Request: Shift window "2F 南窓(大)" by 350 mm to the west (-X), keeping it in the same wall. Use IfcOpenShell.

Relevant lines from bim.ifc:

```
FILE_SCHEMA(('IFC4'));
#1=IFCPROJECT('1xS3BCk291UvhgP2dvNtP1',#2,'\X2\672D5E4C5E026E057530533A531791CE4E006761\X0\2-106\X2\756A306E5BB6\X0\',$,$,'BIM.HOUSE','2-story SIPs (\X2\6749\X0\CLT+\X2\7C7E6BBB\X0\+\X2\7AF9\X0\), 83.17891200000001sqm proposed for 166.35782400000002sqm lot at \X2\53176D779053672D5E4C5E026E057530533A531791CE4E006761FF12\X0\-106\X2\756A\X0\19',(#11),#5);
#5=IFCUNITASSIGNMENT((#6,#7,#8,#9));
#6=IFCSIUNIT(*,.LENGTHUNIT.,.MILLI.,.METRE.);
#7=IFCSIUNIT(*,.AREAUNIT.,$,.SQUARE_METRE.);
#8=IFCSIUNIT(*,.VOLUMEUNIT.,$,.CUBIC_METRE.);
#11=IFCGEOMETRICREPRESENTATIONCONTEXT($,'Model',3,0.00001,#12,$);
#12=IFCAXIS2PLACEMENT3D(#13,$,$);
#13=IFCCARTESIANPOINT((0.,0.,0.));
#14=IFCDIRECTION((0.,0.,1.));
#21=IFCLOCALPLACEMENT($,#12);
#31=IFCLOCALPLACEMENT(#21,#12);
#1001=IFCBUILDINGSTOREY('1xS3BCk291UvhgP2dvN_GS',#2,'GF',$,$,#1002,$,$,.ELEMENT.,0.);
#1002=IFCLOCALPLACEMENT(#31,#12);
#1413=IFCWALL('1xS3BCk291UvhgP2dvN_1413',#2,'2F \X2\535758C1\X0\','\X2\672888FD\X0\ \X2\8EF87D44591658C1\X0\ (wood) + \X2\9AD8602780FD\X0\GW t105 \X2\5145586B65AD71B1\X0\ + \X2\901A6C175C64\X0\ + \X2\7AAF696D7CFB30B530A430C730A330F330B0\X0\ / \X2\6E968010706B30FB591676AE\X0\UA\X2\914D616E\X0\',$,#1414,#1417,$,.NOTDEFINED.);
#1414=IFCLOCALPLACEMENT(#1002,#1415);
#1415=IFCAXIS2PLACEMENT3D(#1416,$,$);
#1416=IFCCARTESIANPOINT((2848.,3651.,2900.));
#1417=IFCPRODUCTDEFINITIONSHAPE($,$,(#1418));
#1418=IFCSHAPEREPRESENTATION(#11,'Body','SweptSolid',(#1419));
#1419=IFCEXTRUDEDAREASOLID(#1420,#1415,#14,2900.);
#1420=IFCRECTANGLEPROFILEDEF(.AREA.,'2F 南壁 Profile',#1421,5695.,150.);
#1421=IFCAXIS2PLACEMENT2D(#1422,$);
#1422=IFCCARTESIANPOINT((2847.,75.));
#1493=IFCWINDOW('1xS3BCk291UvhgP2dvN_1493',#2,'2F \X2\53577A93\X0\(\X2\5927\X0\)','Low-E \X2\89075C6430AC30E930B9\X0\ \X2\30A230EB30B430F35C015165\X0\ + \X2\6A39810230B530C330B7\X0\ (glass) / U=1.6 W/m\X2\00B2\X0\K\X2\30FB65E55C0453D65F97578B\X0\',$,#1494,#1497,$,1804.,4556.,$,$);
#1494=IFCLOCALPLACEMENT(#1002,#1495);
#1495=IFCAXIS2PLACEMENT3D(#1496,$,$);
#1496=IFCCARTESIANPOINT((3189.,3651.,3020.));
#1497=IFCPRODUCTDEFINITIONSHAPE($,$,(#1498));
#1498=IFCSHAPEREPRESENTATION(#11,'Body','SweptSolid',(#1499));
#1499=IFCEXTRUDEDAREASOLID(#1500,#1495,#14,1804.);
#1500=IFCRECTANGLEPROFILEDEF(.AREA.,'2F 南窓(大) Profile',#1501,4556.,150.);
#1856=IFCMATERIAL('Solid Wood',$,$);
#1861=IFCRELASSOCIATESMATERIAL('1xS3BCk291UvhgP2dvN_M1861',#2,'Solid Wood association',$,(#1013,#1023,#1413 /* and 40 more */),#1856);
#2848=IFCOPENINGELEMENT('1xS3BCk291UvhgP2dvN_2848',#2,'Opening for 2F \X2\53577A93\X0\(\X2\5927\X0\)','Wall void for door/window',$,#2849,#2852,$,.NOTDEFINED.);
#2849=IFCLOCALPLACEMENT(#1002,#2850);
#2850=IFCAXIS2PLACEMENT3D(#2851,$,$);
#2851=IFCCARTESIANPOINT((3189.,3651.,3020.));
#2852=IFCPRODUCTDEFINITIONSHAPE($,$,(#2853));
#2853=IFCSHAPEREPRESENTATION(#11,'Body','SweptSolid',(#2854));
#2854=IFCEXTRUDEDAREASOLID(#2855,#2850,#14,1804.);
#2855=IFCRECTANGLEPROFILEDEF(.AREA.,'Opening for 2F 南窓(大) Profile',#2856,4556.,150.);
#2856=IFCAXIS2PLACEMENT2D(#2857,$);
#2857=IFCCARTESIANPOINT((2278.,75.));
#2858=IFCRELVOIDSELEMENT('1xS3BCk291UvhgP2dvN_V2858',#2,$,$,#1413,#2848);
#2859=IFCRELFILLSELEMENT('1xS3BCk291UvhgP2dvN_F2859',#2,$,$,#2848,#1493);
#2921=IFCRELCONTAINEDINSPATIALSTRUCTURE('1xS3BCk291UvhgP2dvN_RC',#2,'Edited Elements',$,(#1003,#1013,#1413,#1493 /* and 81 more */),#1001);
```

```python
import ifcopenshell
import ifcopenshell.api.geometry
import ifcopenshell.util.placement

model = ifcopenshell.open("bim.ifc")

window = model.by_guid("1xS3BCk291UvhgP2dvN_1493")
opening = window.FillsVoids[0].RelatingOpeningElement
wall = opening.VoidsElements[0].RelatingBuildingElement

wall_matrix = ifcopenshell.util.placement.get_local_placement(wall.ObjectPlacement)
shift = wall_matrix[:3, 0] * -350.0
before = ifcopenshell.util.placement.get_local_placement(window.ObjectPlacement)[:3, 3].copy()

# The window is not placed relative to its opening, so move both.
for product in (opening, window):
    matrix = ifcopenshell.util.placement.get_local_placement(product.ObjectPlacement)
    matrix[:3, 3] += shift
    ifcopenshell.api.geometry.edit_object_placement(model, product=product, matrix=matrix, is_si=False)

after = ifcopenshell.util.placement.get_local_placement(window.ObjectPlacement)[:3, 3]
print("window moved by", (after - before).round(3) + 0.0)

model.write("bim_edited.ifc")
```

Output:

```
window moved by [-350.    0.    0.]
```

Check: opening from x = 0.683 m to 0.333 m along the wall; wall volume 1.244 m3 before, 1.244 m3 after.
